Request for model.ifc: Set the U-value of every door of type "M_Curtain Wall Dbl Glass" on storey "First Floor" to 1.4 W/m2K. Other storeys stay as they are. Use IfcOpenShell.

First a look at what the model holds.

```python
import ifcopenshell
import ifcopenshell.util.element

model = ifcopenshell.open("model.ifc")
print(model.schema)
storey = next(s for s in model.by_type("IfcBuildingStorey") if s.Name == "First Floor")
doors = [e for e in ifcopenshell.util.element.get_decomposition(storey) if e.is_a("IfcDoor")]
seen = {}
for e in doors:
    element_type = ifcopenshell.util.element.get_type(e)
    key = (element_type.Name if element_type != e and element_type else None, ifcopenshell.util.element.get_pset(e, "Pset_DoorCommon", "ThermalTransmittance"))
    seen[key] = seen.get(key, 0) + 1
for (name, value), count in sorted(seen.items(), key=str):
    print(count, "x", name, "|", value)
```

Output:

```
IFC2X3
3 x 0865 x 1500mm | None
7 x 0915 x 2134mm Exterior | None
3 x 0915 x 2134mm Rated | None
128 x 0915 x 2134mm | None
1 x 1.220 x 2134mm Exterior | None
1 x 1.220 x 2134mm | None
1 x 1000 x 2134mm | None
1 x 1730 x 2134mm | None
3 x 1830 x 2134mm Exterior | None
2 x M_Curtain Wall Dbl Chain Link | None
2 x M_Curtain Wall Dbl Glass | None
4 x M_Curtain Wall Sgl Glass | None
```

```python
import ifcopenshell
import ifcopenshell.api.pset
import ifcopenshell.util.element

model = ifcopenshell.open("model.ifc")

storey = next(s for s in model.by_type("IfcBuildingStorey") if s.Name == "First Floor")
doors = [e for e in ifcopenshell.util.element.get_decomposition(storey) if e.is_a("IfcDoor")]

count = 0
for e in doors:
    element_type = ifcopenshell.util.element.get_type(e)
    if element_type in (None, e) or element_type.Name != "M_Curtain Wall Dbl Glass":
        continue
    # add_pset returns the element's existing set when there is one.
    pset = ifcopenshell.api.pset.add_pset(model, product=e, name="Pset_DoorCommon")
    ifcopenshell.api.pset.edit_pset(model, pset=pset, properties={"ThermalTransmittance": 1.4})
    count += 1

print(count, "doors updated")

model.write("model-out.ifc")
```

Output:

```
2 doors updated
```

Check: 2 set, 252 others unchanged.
